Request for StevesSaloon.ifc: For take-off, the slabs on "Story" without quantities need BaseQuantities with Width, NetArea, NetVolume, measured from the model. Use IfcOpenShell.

First a look at what the model holds.

```python
import ifcopenshell
import ifcopenshell.util.element
import ifcopenshell.util.unit

model = ifcopenshell.open("StevesSaloon.ifc")
print(model.schema)
for unit_type in ("LENGTHUNIT", "AREAUNIT", "VOLUMEUNIT"):
    print(unit_type, ifcopenshell.util.unit.calculate_unit_scale(model, unit_type))
storey = next(s for s in model.by_type("IfcBuildingStorey") if s.Name == "Story")
slabs = [e for e in ifcopenshell.util.element.get_decomposition(storey) if e.is_a("IfcSlab")]
for e in sorted(slabs, key=lambda e: e.id()):
    print(e.id(), e.is_a(), e.Name, list(ifcopenshell.util.element.get_psets(e, qtos_only=True)), sep=" | ")
```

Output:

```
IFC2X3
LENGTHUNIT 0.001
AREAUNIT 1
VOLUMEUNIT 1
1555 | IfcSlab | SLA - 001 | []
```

```python
import ifcopenshell
import ifcopenshell.api.pset
import ifcopenshell.geom
import ifcopenshell.util.element
import ifcopenshell.util.shape
import ifcopenshell.util.unit

model = ifcopenshell.open("StevesSaloon.ifc")
unit_scale = ifcopenshell.util.unit.calculate_unit_scale(model)
area_scale = ifcopenshell.util.unit.calculate_unit_scale(model, "AREAUNIT")
volume_scale = ifcopenshell.util.unit.calculate_unit_scale(model, "VOLUMEUNIT")
settings = ifcopenshell.geom.settings()

storey = next(s for s in model.by_type("IfcBuildingStorey") if s.Name == "Story")
slabs = [e for e in ifcopenshell.util.element.get_decomposition(storey) if e.is_a("IfcSlab")]

for e in sorted(slabs, key=lambda e: e.id()):
    if ifcopenshell.util.element.get_psets(e, qtos_only=True, should_inherit=False):
        continue
    # Geometry comes back in metres, in the element's own axes.
    shape = ifcopenshell.geom.create_shape(settings, e)
    values = {
        "Width": ifcopenshell.util.shape.get_z(shape.geometry) / unit_scale,
        "NetArea": ifcopenshell.util.shape.get_footprint_area(shape.geometry) / area_scale,
        "NetVolume": ifcopenshell.util.shape.get_volume(shape.geometry) / volume_scale,
    }
    qto = ifcopenshell.api.pset.add_qto(model, product=e, name="BaseQuantities")
    ifcopenshell.api.pset.edit_qto(model, qto=qto, properties=values)
    print(e.id(), {k: round(v, 3) for k, v in values.items()})

model.write("StevesSaloon_v2.ifc")
```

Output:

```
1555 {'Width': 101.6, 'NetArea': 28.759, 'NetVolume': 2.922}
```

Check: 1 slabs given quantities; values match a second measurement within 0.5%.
